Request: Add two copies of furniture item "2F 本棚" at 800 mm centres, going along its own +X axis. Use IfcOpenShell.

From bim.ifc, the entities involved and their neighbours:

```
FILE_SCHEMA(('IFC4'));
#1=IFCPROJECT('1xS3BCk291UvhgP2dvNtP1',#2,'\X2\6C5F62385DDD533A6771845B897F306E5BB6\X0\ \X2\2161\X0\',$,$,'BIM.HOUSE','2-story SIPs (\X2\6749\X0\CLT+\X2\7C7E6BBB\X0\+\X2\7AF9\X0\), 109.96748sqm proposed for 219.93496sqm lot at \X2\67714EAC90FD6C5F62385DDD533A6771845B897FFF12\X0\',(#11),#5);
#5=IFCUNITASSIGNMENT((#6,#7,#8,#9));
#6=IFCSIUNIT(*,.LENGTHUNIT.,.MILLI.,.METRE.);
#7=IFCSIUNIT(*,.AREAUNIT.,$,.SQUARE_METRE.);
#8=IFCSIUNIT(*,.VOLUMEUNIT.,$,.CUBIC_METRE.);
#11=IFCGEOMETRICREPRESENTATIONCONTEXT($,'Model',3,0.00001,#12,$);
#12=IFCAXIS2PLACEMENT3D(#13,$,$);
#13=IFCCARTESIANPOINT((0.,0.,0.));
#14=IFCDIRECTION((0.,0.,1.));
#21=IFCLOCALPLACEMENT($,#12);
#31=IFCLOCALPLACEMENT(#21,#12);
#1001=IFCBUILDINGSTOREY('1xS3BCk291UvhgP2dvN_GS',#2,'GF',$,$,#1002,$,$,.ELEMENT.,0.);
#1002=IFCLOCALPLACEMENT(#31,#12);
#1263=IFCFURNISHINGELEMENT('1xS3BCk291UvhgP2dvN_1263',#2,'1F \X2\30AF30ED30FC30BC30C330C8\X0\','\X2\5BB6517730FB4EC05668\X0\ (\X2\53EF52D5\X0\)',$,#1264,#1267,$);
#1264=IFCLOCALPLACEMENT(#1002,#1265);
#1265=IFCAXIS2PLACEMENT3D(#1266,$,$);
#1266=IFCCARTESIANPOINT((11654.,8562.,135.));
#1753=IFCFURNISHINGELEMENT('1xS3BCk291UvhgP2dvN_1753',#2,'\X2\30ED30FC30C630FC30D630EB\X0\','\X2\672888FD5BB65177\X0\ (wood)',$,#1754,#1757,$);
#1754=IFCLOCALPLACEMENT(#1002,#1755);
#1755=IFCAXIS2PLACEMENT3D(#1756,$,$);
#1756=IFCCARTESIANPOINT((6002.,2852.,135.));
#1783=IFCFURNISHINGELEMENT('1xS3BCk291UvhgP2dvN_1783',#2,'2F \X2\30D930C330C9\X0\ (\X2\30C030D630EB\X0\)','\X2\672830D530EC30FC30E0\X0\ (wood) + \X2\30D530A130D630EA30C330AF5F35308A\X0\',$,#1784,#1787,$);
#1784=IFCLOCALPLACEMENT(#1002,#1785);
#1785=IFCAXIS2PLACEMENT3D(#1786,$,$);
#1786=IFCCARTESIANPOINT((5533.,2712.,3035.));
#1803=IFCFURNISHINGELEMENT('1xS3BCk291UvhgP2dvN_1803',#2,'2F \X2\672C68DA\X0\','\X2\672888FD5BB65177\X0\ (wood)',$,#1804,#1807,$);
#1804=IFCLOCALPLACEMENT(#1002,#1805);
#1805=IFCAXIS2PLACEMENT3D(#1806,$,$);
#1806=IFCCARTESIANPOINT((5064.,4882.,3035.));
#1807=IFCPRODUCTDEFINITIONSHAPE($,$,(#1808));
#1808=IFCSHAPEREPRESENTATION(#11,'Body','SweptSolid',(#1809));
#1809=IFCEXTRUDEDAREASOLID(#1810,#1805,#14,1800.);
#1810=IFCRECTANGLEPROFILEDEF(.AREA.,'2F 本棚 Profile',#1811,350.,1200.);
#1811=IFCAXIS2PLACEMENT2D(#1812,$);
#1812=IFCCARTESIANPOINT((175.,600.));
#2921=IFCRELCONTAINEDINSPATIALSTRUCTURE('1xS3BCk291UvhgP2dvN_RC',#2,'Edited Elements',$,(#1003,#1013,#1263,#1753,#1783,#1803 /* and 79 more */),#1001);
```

```python
import ifcopenshell
import ifcopenshell.api.geometry
import ifcopenshell.api.root
import ifcopenshell.util.element
import ifcopenshell.util.placement

model = ifcopenshell.open("bim.ifc")


def reuse_history(source, copy):
    """copy_class also copies each property set's owner history, people and application; keep the originals."""
    for rel in copy.IsDefinedBy:
        if rel.is_a("IfcRelDefinesByProperties") and (history := rel.RelatingPropertyDefinition.OwnerHistory):
            rel.RelatingPropertyDefinition.OwnerHistory = source.OwnerHistory
            ifcopenshell.util.element.remove_deep2(model, history)


source = model.by_guid("1xS3BCk291UvhgP2dvN_1803")
base = ifcopenshell.util.placement.get_local_placement(source.ObjectPlacement)
step = base[:3, 0] * 800.0

for i in range(1, 3):
    copy = ifcopenshell.api.root.copy_class(model, product=source)
    copy.Representation = ifcopenshell.util.element.copy_deep(
        model, source.Representation, exclude=["IfcGeometricRepresentationContext", "IfcRepresentationMap"]
    )
    reuse_history(source, copy)
    matrix = base.copy()
    matrix[:3, 3] += i * step
    print("added at", matrix[:3, 3].round(3) + 0.0)
    ifcopenshell.api.geometry.edit_object_placement(model, product=copy, matrix=matrix, is_si=False)

model.write("bim_v2.ifc")
```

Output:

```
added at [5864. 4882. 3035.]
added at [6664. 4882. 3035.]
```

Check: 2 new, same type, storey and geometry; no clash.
